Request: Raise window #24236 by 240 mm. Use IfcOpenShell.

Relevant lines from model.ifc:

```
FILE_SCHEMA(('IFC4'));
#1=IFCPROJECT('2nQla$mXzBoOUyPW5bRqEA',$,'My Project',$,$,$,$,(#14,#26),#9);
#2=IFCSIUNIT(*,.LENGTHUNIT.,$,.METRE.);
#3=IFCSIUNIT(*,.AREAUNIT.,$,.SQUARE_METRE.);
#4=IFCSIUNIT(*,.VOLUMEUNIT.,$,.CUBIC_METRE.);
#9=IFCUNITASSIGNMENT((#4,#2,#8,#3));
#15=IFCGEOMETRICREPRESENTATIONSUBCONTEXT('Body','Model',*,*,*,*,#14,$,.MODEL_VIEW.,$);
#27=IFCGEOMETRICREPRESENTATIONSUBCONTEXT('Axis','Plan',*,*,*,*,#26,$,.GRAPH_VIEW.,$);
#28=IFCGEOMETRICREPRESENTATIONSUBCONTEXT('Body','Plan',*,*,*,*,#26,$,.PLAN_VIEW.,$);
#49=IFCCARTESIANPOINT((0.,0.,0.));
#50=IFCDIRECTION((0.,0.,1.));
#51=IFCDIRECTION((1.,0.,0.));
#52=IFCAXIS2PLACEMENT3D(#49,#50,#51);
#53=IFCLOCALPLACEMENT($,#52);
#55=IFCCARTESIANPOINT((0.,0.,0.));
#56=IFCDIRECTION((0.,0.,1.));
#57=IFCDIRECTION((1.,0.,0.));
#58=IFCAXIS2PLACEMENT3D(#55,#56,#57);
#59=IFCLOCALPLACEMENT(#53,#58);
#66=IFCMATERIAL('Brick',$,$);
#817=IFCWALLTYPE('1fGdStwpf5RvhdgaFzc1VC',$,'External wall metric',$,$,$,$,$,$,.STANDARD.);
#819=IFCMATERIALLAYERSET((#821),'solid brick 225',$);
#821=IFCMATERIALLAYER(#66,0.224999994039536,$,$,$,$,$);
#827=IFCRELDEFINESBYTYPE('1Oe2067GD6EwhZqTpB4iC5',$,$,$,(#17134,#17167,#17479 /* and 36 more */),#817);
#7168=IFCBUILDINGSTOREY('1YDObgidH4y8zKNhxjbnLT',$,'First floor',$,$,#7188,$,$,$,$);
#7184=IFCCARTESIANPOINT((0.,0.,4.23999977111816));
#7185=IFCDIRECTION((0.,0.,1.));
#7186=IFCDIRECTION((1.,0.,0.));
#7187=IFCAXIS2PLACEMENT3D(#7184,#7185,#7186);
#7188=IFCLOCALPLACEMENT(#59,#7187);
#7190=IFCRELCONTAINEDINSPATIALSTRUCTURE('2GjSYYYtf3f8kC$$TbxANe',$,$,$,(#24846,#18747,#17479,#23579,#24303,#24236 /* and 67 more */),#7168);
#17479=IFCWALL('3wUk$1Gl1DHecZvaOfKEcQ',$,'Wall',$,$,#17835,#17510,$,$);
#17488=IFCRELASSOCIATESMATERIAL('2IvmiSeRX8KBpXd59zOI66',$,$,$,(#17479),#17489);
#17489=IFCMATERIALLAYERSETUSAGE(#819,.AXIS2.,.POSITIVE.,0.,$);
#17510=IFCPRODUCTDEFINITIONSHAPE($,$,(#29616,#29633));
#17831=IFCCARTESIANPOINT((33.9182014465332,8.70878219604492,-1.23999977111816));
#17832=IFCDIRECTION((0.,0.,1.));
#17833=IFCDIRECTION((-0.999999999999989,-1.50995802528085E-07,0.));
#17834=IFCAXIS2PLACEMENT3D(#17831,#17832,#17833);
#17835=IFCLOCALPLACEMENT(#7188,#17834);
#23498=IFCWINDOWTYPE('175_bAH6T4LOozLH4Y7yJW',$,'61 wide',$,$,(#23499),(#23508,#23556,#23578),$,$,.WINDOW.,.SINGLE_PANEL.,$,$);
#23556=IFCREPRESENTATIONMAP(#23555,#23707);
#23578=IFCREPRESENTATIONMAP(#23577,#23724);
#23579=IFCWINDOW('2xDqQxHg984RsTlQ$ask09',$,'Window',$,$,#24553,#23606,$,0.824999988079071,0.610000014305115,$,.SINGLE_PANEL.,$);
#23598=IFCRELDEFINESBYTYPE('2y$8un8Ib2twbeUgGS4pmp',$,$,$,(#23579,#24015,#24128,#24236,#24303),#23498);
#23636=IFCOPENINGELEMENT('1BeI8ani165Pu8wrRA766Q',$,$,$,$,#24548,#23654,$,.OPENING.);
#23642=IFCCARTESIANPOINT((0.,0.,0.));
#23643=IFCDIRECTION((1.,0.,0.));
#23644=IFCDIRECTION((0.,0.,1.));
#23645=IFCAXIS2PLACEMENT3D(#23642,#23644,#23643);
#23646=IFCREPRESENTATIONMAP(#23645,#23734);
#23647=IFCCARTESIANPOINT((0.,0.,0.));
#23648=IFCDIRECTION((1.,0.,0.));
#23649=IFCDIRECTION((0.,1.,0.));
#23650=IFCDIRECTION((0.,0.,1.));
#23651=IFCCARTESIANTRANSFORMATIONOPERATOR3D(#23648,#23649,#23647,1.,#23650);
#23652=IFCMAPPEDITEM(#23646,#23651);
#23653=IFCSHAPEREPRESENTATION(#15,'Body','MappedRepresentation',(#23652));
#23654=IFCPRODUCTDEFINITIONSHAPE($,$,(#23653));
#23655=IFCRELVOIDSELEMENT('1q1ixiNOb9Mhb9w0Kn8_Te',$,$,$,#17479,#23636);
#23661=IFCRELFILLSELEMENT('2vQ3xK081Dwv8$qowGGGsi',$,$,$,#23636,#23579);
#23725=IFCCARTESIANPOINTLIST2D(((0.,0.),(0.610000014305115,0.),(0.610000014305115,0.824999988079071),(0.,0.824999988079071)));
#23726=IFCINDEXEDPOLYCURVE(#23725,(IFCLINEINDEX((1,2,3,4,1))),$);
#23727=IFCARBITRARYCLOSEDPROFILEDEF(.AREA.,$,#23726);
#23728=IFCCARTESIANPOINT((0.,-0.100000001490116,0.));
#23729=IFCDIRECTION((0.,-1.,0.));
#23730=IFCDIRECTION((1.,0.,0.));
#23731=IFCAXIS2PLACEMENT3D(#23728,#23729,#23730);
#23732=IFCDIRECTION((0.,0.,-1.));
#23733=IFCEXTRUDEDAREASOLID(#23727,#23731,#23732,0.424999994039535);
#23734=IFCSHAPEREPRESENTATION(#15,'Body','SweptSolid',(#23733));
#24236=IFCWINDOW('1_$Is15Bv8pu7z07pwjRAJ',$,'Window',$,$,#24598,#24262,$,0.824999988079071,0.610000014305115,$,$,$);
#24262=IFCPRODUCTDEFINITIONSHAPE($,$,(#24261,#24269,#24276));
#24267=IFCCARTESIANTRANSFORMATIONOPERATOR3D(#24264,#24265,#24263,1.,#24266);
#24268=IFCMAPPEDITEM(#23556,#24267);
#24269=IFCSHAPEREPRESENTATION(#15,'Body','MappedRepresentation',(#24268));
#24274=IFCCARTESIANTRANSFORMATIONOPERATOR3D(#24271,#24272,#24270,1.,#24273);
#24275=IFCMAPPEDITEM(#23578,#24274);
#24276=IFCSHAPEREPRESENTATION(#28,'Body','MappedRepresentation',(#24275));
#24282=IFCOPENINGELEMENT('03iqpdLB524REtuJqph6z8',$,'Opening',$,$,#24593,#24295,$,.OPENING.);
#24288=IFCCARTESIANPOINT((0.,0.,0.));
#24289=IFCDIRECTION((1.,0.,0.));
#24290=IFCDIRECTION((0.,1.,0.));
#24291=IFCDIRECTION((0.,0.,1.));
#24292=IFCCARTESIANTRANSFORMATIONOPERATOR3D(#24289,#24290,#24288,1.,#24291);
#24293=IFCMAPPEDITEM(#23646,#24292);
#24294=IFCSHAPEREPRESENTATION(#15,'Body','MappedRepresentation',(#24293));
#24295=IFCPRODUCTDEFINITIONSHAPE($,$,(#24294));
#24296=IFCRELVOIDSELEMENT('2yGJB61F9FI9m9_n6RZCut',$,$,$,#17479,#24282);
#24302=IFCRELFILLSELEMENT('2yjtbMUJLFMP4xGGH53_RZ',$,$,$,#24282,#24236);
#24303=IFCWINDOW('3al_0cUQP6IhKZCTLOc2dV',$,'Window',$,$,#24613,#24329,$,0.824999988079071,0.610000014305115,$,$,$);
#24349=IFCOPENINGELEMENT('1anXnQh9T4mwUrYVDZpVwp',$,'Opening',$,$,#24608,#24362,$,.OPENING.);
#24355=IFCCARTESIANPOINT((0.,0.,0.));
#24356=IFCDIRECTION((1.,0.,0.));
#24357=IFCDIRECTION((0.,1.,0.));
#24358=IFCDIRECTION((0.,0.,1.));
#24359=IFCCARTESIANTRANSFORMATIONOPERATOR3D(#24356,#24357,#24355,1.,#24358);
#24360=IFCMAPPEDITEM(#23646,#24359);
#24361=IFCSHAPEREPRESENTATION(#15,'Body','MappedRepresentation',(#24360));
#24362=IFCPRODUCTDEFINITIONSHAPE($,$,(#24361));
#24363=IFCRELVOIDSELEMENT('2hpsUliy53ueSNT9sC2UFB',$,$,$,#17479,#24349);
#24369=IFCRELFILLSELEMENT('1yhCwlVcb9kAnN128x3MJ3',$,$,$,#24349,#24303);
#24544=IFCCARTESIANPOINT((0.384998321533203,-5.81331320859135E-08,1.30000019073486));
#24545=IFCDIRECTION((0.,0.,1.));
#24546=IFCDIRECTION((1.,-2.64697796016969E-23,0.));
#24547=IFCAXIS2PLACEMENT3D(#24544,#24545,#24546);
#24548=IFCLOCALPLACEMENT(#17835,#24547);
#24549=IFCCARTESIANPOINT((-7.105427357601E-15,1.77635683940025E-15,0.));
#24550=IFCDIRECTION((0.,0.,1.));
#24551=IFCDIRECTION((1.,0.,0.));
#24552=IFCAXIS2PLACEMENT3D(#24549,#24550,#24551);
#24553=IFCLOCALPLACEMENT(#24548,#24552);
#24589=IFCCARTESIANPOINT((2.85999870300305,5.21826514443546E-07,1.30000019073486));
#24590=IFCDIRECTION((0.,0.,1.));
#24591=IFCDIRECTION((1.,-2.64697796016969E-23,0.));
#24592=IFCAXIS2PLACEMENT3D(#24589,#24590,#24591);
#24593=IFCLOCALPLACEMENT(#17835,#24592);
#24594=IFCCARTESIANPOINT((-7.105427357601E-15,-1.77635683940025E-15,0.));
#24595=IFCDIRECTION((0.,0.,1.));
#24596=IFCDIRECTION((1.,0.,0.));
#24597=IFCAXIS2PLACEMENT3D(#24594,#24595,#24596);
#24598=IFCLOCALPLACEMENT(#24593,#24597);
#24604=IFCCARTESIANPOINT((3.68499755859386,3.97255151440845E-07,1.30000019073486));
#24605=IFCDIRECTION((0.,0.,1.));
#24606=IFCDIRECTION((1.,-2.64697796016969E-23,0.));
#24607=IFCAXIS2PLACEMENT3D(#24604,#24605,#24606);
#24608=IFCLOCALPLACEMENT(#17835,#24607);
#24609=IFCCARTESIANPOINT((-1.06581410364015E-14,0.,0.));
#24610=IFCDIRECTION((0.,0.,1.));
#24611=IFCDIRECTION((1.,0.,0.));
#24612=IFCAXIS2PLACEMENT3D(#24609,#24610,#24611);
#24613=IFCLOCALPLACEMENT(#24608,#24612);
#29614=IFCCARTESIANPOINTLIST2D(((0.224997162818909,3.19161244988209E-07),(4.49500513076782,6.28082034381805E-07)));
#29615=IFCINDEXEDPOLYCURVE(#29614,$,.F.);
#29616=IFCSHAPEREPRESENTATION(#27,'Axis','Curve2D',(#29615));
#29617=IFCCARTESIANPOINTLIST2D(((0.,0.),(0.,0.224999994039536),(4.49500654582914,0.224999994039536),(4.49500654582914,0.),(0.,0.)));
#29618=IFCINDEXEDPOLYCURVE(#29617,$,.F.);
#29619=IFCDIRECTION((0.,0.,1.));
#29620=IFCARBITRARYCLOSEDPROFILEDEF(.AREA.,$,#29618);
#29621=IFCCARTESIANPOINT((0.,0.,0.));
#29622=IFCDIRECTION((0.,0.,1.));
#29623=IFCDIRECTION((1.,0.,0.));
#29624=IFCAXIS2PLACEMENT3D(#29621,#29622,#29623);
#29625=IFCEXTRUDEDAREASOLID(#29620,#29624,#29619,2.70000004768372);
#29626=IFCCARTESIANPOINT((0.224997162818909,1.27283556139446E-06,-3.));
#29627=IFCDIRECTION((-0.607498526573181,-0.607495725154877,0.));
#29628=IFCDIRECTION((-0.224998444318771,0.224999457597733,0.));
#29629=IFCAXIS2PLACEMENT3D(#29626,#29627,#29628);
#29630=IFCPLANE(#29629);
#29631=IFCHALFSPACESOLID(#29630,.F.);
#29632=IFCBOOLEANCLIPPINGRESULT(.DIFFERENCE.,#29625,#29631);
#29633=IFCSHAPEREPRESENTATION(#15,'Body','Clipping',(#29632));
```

```python
import numpy as np
import ifcopenshell
import ifcopenshell.api.geometry
import ifcopenshell.util.placement
import ifcopenshell.util.unit

model = ifcopenshell.open("model.ifc")
unit_scale = ifcopenshell.util.unit.calculate_unit_scale(model)

window = model.by_id(24236)
opening = window.FillsVoids[0].RelatingOpeningElement
dz = 0.24 / unit_scale

shift = np.array([0.0, 0.0, dz])
# The window is placed relative to its opening, so it follows when the opening moves.
matrix = ifcopenshell.util.placement.get_local_placement(opening.ObjectPlacement)
matrix[:3, 3] += shift
ifcopenshell.api.geometry.edit_object_placement(
    model, product=opening, matrix=matrix, is_si=False, should_transform_children=True
)

print(f"moved by {dz * unit_scale:+.3f} m")

model.write("model_v2.ifc")
```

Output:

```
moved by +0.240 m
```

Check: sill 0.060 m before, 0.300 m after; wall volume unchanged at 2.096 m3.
